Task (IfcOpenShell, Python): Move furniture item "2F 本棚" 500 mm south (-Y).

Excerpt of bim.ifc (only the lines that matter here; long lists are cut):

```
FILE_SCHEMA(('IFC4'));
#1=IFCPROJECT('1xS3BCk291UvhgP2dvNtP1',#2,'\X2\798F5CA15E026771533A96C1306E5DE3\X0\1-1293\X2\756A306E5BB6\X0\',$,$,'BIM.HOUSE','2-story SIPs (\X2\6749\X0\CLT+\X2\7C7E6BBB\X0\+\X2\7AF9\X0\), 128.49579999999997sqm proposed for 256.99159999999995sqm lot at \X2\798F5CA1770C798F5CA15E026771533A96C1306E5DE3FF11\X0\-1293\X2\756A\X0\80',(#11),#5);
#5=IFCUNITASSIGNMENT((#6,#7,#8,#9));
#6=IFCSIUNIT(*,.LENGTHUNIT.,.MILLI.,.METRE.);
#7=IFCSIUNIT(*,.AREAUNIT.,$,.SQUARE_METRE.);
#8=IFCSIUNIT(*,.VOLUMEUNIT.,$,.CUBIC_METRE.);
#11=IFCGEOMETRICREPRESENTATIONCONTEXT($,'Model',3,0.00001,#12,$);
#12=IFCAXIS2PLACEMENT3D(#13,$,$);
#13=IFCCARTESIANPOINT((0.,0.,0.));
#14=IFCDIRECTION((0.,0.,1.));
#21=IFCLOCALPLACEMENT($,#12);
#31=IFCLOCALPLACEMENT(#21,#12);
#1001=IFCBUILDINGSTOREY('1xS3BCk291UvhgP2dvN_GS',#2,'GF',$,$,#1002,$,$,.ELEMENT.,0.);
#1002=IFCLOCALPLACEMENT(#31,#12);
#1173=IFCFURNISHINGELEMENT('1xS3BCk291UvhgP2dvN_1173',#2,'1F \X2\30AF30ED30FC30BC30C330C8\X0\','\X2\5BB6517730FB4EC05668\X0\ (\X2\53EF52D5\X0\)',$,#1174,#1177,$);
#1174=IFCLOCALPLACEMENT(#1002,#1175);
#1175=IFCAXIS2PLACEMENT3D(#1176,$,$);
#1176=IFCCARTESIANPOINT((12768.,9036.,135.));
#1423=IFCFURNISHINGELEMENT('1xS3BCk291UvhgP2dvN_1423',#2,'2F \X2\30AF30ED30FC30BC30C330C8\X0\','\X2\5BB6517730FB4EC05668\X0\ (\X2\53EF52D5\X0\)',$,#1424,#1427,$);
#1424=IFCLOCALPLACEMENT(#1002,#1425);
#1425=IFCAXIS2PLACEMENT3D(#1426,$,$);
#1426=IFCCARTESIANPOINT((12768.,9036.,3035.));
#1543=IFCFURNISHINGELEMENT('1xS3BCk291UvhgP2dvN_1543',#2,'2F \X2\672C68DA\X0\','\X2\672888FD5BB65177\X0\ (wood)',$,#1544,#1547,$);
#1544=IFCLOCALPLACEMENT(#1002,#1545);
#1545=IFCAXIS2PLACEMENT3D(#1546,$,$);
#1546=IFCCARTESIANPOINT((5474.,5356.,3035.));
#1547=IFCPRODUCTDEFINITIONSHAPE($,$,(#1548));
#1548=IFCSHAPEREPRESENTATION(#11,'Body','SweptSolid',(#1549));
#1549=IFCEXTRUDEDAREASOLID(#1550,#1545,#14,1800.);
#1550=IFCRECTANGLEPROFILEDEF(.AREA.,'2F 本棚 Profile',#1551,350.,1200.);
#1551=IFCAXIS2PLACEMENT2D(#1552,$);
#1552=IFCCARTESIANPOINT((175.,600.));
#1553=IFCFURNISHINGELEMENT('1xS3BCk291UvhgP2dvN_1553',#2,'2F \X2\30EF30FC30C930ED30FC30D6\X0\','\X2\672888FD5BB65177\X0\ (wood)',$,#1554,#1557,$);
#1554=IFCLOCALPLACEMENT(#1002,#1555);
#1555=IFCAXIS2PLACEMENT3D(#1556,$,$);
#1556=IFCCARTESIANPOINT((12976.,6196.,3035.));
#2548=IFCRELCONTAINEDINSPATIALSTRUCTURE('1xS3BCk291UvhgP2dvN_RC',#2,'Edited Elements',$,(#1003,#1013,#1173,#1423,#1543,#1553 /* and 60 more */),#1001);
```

```python
import ifcopenshell
import ifcopenshell.api.geometry
import ifcopenshell.util.placement
import ifcopenshell.util.unit

model = ifcopenshell.open("bim.ifc")
unit_scale = ifcopenshell.util.unit.calculate_unit_scale(model)

item = model.by_guid("1xS3BCk291UvhgP2dvN_1543")
matrix = ifcopenshell.util.placement.get_local_placement(item.ObjectPlacement)
matrix[1, 3] -= 0.5 / unit_scale
ifcopenshell.api.geometry.edit_object_placement(model, product=item, matrix=matrix, is_si=False)

print(ifcopenshell.util.placement.get_local_placement(item.ObjectPlacement).round(3) + 0.0)

model.write("bim_rev.ifc")
```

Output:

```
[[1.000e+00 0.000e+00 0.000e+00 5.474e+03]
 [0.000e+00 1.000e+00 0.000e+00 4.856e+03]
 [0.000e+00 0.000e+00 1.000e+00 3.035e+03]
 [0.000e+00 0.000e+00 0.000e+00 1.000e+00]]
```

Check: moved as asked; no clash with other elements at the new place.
